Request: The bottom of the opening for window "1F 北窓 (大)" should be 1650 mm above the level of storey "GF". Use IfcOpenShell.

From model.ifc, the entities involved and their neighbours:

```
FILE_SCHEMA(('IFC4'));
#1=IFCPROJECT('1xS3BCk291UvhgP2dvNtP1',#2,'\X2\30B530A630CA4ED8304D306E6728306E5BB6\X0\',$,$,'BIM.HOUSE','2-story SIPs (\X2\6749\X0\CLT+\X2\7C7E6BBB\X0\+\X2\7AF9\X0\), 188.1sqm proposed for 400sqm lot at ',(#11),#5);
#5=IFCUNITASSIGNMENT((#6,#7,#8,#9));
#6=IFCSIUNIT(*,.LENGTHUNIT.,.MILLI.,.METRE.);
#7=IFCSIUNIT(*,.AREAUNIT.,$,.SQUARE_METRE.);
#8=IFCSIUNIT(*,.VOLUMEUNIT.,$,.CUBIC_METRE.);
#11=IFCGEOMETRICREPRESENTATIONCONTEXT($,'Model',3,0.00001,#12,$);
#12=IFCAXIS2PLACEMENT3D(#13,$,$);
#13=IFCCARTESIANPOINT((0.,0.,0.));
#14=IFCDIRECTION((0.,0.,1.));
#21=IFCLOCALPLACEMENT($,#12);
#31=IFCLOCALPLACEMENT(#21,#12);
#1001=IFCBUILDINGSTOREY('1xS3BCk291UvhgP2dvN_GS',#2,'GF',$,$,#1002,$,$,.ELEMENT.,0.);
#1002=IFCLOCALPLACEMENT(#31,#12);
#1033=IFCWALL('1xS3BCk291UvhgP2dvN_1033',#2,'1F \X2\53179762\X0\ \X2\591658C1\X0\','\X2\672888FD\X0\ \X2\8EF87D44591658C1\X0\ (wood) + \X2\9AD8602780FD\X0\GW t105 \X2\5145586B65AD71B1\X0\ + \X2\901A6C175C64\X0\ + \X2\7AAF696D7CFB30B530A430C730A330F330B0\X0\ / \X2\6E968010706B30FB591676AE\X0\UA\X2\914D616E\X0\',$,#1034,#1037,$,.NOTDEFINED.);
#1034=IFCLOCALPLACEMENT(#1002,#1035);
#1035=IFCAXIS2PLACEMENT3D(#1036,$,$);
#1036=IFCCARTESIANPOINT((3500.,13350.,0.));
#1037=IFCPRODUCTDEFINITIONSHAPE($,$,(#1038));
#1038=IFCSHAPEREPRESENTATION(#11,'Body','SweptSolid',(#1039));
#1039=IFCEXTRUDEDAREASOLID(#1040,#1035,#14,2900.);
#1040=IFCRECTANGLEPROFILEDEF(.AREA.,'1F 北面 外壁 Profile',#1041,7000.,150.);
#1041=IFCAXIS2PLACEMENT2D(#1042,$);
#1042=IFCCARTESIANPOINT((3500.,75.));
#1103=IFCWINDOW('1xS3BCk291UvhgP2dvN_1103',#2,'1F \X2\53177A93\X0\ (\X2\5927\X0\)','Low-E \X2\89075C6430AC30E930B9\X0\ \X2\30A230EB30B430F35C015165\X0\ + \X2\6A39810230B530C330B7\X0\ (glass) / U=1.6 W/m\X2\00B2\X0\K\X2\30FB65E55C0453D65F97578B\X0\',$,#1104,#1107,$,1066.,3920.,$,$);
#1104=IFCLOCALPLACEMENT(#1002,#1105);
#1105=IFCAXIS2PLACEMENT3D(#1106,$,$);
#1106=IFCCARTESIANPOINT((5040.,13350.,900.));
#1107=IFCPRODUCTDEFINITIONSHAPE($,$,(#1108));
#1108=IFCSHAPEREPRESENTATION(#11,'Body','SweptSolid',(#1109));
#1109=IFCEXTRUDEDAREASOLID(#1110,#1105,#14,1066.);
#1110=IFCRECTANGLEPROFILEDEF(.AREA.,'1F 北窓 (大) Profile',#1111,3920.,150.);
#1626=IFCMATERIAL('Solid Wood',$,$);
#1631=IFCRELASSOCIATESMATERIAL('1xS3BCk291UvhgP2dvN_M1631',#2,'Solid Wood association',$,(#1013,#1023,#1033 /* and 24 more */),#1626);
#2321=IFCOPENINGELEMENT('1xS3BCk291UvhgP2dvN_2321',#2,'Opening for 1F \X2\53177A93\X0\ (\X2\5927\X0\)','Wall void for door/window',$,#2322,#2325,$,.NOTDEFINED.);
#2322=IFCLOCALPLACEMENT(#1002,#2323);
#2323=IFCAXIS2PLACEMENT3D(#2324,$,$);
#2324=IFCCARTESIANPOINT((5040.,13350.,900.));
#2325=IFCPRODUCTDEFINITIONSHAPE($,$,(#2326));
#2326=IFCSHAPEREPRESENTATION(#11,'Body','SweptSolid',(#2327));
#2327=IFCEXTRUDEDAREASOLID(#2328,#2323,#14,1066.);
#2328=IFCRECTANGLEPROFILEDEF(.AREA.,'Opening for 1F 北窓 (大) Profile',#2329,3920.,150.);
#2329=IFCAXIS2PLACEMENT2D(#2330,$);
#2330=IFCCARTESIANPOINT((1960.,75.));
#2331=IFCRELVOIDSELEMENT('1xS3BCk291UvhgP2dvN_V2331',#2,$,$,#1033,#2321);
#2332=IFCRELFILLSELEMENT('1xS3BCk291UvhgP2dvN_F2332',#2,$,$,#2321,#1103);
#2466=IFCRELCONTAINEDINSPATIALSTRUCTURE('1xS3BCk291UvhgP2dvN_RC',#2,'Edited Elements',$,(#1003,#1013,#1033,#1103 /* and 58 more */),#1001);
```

```python
import numpy as np
import ifcopenshell
import ifcopenshell.api.geometry
import ifcopenshell.geom
import ifcopenshell.util.element
import ifcopenshell.util.placement
import ifcopenshell.util.shape
import ifcopenshell.util.unit

model = ifcopenshell.open("model.ifc")
unit_scale = ifcopenshell.util.unit.calculate_unit_scale(model)

window = model.by_guid("1xS3BCk291UvhgP2dvN_1103")
opening = window.FillsVoids[0].RelatingOpeningElement
storey = ifcopenshell.util.element.get_container(window, ifc_class="IfcBuildingStorey")
level = ifcopenshell.util.placement.get_local_placement(storey.ObjectPlacement)[2, 3]

# The opening's origin need not be at the sill, so measure its lowest point.
shape = ifcopenshell.geom.create_shape(ifcopenshell.geom.settings(), opening)
bottom = ifcopenshell.util.shape.get_shape_bottom_elevation(shape, shape.geometry) / unit_scale
dz = level + 1.65 / unit_scale - bottom

shift = np.array([0.0, 0.0, dz])
# The window is not placed relative to its opening, so move both.
for product in (opening, window):
    matrix = ifcopenshell.util.placement.get_local_placement(product.ObjectPlacement)
    matrix[:3, 3] += shift
    ifcopenshell.api.geometry.edit_object_placement(model, product=product, matrix=matrix, is_si=False)

print(f"moved by {dz * unit_scale:+.3f} m")

model.write("model_edited.ifc")
```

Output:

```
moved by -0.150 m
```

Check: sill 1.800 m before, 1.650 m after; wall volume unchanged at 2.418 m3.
